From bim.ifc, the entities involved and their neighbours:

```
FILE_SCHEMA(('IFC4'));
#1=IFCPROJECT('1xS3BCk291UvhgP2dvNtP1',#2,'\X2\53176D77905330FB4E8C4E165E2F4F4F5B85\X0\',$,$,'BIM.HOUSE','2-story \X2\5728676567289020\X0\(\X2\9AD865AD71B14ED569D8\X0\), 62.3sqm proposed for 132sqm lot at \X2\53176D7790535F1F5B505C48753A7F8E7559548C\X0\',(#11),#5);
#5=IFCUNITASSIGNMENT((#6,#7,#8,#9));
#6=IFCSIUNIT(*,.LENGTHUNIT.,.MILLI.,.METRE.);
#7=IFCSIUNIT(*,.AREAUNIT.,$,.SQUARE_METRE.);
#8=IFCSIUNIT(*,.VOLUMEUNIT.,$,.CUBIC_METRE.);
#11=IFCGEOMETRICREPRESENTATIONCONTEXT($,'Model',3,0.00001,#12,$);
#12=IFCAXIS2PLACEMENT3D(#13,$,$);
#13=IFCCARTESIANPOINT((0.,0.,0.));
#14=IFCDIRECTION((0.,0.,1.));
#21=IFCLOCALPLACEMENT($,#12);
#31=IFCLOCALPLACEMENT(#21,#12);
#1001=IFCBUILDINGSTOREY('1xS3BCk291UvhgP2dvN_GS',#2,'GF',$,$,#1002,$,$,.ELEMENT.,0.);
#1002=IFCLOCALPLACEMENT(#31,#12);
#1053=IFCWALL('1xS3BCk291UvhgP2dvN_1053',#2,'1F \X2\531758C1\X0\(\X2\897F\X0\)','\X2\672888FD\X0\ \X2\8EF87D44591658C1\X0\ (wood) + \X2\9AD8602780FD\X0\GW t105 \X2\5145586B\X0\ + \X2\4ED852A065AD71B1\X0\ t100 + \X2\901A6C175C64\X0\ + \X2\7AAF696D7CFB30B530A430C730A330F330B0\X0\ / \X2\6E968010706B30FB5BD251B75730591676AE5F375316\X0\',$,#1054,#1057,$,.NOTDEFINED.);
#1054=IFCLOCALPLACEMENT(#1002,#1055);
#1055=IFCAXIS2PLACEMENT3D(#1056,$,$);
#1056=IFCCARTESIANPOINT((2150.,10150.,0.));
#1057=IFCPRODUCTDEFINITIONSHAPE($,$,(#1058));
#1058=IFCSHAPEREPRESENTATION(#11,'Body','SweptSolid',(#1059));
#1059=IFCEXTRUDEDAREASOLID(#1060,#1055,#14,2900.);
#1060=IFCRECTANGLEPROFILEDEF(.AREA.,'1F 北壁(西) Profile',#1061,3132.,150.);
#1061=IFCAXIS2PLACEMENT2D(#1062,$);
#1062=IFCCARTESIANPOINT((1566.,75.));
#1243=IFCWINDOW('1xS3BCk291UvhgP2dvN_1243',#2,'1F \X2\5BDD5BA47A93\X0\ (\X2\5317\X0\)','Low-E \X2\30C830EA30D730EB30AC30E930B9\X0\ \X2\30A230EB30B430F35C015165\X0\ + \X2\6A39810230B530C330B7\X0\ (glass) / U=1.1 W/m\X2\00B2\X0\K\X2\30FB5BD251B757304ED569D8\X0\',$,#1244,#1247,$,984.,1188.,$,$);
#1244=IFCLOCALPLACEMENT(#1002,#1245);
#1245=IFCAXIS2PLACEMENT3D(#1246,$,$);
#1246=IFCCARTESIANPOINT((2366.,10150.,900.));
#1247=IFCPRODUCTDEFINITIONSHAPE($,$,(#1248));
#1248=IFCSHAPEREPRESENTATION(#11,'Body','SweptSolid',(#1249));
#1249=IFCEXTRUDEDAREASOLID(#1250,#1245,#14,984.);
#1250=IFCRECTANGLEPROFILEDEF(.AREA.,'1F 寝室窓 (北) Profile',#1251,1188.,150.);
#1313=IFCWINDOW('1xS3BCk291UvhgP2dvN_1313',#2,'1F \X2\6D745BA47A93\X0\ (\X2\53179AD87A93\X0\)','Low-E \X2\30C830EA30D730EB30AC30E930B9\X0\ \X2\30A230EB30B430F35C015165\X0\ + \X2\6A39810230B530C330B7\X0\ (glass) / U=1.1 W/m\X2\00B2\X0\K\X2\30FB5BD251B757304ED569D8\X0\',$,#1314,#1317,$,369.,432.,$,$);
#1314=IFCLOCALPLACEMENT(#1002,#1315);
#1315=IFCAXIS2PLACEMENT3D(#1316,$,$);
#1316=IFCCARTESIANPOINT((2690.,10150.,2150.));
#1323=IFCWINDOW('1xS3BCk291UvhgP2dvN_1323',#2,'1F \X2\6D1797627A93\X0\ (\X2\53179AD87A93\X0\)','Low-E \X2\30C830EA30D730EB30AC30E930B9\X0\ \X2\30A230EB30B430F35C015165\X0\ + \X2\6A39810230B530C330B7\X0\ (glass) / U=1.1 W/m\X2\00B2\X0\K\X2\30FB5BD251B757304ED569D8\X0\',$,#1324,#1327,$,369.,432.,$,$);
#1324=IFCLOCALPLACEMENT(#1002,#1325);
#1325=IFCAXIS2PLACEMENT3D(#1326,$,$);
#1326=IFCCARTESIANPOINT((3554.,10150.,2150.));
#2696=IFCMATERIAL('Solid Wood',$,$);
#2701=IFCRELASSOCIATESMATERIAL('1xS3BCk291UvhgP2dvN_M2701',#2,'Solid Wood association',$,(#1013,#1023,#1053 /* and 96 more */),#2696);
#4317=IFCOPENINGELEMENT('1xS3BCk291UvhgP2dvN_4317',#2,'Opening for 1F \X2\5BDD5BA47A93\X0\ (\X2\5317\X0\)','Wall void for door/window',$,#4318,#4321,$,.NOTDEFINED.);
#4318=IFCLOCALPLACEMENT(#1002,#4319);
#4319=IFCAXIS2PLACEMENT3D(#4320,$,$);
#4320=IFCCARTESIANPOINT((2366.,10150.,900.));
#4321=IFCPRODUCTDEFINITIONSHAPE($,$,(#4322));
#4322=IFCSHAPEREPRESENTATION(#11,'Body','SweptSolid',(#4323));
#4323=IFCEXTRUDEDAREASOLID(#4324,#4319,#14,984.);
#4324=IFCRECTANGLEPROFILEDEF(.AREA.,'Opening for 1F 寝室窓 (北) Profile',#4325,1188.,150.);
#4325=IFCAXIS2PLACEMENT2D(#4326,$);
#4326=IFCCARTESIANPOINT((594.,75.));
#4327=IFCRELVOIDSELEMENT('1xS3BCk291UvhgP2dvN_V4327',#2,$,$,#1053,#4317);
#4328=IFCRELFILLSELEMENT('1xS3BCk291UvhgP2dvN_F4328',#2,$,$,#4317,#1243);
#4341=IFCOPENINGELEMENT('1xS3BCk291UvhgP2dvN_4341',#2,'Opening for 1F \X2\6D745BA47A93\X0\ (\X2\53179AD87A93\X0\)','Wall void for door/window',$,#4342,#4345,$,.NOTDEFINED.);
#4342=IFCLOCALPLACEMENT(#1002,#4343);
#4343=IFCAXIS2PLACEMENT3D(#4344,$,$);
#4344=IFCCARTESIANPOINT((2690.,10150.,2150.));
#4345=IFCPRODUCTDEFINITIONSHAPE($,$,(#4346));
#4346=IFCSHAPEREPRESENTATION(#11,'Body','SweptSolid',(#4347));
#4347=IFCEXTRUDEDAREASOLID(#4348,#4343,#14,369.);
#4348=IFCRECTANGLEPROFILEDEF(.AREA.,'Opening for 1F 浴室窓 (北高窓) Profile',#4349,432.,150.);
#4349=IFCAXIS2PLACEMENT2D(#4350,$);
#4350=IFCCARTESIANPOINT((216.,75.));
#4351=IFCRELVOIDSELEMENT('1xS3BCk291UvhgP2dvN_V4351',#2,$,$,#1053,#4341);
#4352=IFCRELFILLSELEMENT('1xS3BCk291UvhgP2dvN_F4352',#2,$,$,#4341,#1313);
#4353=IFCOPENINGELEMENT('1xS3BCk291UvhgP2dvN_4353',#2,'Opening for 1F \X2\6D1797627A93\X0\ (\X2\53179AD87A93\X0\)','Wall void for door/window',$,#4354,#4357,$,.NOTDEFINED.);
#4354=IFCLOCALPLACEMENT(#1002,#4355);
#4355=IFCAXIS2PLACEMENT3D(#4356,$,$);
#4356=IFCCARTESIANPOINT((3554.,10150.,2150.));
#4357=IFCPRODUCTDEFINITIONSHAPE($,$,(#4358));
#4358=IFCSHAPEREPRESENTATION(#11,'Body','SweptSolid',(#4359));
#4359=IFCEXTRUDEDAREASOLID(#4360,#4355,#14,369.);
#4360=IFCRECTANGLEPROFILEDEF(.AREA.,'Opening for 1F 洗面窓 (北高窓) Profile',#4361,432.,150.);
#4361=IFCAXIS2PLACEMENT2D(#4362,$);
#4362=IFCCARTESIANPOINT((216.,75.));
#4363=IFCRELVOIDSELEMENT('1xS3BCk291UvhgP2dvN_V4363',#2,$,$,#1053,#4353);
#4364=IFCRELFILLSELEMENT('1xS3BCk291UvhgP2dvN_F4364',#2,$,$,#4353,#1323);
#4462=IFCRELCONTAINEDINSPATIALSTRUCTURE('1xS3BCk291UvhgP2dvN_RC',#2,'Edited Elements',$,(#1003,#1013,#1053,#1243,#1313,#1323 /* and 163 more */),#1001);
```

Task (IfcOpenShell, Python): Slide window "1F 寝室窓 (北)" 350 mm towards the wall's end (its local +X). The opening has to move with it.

```python
import ifcopenshell
import ifcopenshell.api.geometry
import ifcopenshell.util.placement

model = ifcopenshell.open("bim.ifc")

window = model.by_guid("1xS3BCk291UvhgP2dvN_1243")
opening = window.FillsVoids[0].RelatingOpeningElement
wall = opening.VoidsElements[0].RelatingBuildingElement

wall_matrix = ifcopenshell.util.placement.get_local_placement(wall.ObjectPlacement)
shift = wall_matrix[:3, 0] * 350.0
before = ifcopenshell.util.placement.get_local_placement(window.ObjectPlacement)[:3, 3].copy()

# The window is not placed relative to its opening, so move both.
for product in (opening, window):
    matrix = ifcopenshell.util.placement.get_local_placement(product.ObjectPlacement)
    matrix[:3, 3] += shift
    ifcopenshell.api.geometry.edit_object_placement(model, product=product, matrix=matrix, is_si=False)

after = ifcopenshell.util.placement.get_local_placement(window.ObjectPlacement)[:3, 3]
print("window moved by", (after - before).round(3) + 0.0)

model.write("bim_rev.ifc")
```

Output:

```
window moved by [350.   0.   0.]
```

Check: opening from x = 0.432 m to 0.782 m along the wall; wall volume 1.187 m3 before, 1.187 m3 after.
